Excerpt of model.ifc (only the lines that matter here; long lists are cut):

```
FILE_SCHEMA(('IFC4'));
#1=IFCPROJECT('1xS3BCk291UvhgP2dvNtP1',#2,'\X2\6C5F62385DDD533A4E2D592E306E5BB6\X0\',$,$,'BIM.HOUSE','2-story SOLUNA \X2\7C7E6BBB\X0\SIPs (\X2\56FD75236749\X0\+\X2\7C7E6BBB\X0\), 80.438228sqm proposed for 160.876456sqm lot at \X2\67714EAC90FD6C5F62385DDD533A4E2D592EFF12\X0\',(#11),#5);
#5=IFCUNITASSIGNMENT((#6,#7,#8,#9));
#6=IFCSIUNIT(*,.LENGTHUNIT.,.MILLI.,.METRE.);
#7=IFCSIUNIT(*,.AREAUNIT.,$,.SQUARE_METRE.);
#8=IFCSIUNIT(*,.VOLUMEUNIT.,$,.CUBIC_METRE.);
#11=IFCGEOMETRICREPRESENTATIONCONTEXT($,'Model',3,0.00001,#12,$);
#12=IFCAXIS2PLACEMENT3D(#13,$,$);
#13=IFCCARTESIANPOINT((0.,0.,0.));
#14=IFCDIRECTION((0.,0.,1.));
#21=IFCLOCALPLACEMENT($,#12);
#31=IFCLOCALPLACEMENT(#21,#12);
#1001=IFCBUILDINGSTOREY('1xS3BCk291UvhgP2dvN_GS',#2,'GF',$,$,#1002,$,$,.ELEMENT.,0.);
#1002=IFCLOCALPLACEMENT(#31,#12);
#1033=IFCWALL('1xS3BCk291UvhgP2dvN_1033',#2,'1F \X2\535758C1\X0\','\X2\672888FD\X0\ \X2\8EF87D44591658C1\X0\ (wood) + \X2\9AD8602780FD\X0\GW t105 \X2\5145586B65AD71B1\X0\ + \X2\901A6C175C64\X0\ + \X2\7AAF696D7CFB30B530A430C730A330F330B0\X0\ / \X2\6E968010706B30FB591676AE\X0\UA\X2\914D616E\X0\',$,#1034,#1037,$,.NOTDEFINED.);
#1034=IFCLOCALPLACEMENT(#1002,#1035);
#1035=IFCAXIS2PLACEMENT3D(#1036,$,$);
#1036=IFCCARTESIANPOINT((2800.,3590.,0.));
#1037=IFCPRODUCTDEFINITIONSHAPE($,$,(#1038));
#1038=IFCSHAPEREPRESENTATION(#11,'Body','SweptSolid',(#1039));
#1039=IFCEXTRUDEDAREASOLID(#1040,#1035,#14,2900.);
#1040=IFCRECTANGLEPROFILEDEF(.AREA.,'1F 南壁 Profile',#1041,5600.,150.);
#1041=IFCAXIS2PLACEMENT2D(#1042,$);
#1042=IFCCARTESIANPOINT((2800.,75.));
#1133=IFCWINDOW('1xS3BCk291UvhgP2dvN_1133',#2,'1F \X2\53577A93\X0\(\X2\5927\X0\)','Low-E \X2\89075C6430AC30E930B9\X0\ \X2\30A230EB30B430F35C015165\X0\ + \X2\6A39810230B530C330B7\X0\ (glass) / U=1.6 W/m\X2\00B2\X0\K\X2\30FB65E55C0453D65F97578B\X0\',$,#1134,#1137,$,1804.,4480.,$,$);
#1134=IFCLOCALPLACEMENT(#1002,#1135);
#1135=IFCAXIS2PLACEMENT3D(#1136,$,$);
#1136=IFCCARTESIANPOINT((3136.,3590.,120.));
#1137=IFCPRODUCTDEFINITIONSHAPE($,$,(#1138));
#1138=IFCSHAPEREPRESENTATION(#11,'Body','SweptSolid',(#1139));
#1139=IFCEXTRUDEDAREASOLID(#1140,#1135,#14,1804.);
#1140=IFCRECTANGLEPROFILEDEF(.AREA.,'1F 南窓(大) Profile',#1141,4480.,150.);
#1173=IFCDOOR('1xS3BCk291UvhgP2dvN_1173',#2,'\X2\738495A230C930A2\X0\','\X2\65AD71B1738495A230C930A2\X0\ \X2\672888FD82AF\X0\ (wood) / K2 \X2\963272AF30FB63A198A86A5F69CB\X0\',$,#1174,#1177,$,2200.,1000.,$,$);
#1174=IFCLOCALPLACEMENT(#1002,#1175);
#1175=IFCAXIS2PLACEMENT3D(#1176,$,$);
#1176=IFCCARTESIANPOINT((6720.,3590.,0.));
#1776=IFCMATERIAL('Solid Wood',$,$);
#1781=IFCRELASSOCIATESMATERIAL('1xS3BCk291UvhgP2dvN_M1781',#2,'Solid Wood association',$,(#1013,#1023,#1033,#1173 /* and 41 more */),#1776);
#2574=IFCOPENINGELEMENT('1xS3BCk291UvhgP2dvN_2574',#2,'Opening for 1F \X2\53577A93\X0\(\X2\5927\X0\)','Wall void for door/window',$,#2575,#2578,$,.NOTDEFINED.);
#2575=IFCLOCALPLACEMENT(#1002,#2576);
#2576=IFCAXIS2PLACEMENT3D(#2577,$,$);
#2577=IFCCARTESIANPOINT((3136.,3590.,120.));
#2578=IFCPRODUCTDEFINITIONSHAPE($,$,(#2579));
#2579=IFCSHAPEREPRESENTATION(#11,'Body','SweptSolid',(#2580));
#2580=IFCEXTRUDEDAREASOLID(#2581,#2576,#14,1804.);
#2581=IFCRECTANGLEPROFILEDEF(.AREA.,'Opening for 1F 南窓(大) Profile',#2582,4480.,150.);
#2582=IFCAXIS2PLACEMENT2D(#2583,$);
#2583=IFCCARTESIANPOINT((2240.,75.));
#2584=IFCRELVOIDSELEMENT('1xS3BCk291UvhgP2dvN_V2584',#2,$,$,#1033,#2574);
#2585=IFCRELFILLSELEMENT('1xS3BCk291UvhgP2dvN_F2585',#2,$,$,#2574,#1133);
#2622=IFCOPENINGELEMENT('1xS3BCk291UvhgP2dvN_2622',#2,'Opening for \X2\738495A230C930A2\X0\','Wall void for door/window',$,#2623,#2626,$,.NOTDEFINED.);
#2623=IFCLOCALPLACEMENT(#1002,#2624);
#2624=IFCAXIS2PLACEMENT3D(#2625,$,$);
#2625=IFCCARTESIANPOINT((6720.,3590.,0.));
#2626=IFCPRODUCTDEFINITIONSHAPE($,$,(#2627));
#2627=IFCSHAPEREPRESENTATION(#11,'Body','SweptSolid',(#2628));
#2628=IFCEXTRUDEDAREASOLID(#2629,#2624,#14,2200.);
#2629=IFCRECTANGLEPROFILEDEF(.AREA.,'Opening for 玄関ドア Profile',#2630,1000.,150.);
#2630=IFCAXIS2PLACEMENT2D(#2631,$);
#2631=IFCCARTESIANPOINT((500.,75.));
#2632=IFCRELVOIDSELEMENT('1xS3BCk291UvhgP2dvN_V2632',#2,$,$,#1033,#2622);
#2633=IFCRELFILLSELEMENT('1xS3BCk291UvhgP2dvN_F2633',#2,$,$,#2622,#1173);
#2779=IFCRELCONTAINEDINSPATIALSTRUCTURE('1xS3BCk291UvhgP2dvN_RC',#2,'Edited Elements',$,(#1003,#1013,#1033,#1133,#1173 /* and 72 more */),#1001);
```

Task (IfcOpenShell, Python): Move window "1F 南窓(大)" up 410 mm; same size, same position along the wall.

```python
import numpy as np
import ifcopenshell
import ifcopenshell.api.geometry
import ifcopenshell.util.placement
import ifcopenshell.util.unit

model = ifcopenshell.open("model.ifc")
unit_scale = ifcopenshell.util.unit.calculate_unit_scale(model)

window = model.by_guid("1xS3BCk291UvhgP2dvN_1133")
opening = window.FillsVoids[0].RelatingOpeningElement
dz = 0.41 / unit_scale

shift = np.array([0.0, 0.0, dz])
# The window is not placed relative to its opening, so move both.
for product in (opening, window):
    matrix = ifcopenshell.util.placement.get_local_placement(product.ObjectPlacement)
    matrix[:3, 3] += shift
    ifcopenshell.api.geometry.edit_object_placement(model, product=product, matrix=matrix, is_si=False)

print(f"moved by {dz * unit_scale:+.3f} m")

model.write("model_updated.ifc")
```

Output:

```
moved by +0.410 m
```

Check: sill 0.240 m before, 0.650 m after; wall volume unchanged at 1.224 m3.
